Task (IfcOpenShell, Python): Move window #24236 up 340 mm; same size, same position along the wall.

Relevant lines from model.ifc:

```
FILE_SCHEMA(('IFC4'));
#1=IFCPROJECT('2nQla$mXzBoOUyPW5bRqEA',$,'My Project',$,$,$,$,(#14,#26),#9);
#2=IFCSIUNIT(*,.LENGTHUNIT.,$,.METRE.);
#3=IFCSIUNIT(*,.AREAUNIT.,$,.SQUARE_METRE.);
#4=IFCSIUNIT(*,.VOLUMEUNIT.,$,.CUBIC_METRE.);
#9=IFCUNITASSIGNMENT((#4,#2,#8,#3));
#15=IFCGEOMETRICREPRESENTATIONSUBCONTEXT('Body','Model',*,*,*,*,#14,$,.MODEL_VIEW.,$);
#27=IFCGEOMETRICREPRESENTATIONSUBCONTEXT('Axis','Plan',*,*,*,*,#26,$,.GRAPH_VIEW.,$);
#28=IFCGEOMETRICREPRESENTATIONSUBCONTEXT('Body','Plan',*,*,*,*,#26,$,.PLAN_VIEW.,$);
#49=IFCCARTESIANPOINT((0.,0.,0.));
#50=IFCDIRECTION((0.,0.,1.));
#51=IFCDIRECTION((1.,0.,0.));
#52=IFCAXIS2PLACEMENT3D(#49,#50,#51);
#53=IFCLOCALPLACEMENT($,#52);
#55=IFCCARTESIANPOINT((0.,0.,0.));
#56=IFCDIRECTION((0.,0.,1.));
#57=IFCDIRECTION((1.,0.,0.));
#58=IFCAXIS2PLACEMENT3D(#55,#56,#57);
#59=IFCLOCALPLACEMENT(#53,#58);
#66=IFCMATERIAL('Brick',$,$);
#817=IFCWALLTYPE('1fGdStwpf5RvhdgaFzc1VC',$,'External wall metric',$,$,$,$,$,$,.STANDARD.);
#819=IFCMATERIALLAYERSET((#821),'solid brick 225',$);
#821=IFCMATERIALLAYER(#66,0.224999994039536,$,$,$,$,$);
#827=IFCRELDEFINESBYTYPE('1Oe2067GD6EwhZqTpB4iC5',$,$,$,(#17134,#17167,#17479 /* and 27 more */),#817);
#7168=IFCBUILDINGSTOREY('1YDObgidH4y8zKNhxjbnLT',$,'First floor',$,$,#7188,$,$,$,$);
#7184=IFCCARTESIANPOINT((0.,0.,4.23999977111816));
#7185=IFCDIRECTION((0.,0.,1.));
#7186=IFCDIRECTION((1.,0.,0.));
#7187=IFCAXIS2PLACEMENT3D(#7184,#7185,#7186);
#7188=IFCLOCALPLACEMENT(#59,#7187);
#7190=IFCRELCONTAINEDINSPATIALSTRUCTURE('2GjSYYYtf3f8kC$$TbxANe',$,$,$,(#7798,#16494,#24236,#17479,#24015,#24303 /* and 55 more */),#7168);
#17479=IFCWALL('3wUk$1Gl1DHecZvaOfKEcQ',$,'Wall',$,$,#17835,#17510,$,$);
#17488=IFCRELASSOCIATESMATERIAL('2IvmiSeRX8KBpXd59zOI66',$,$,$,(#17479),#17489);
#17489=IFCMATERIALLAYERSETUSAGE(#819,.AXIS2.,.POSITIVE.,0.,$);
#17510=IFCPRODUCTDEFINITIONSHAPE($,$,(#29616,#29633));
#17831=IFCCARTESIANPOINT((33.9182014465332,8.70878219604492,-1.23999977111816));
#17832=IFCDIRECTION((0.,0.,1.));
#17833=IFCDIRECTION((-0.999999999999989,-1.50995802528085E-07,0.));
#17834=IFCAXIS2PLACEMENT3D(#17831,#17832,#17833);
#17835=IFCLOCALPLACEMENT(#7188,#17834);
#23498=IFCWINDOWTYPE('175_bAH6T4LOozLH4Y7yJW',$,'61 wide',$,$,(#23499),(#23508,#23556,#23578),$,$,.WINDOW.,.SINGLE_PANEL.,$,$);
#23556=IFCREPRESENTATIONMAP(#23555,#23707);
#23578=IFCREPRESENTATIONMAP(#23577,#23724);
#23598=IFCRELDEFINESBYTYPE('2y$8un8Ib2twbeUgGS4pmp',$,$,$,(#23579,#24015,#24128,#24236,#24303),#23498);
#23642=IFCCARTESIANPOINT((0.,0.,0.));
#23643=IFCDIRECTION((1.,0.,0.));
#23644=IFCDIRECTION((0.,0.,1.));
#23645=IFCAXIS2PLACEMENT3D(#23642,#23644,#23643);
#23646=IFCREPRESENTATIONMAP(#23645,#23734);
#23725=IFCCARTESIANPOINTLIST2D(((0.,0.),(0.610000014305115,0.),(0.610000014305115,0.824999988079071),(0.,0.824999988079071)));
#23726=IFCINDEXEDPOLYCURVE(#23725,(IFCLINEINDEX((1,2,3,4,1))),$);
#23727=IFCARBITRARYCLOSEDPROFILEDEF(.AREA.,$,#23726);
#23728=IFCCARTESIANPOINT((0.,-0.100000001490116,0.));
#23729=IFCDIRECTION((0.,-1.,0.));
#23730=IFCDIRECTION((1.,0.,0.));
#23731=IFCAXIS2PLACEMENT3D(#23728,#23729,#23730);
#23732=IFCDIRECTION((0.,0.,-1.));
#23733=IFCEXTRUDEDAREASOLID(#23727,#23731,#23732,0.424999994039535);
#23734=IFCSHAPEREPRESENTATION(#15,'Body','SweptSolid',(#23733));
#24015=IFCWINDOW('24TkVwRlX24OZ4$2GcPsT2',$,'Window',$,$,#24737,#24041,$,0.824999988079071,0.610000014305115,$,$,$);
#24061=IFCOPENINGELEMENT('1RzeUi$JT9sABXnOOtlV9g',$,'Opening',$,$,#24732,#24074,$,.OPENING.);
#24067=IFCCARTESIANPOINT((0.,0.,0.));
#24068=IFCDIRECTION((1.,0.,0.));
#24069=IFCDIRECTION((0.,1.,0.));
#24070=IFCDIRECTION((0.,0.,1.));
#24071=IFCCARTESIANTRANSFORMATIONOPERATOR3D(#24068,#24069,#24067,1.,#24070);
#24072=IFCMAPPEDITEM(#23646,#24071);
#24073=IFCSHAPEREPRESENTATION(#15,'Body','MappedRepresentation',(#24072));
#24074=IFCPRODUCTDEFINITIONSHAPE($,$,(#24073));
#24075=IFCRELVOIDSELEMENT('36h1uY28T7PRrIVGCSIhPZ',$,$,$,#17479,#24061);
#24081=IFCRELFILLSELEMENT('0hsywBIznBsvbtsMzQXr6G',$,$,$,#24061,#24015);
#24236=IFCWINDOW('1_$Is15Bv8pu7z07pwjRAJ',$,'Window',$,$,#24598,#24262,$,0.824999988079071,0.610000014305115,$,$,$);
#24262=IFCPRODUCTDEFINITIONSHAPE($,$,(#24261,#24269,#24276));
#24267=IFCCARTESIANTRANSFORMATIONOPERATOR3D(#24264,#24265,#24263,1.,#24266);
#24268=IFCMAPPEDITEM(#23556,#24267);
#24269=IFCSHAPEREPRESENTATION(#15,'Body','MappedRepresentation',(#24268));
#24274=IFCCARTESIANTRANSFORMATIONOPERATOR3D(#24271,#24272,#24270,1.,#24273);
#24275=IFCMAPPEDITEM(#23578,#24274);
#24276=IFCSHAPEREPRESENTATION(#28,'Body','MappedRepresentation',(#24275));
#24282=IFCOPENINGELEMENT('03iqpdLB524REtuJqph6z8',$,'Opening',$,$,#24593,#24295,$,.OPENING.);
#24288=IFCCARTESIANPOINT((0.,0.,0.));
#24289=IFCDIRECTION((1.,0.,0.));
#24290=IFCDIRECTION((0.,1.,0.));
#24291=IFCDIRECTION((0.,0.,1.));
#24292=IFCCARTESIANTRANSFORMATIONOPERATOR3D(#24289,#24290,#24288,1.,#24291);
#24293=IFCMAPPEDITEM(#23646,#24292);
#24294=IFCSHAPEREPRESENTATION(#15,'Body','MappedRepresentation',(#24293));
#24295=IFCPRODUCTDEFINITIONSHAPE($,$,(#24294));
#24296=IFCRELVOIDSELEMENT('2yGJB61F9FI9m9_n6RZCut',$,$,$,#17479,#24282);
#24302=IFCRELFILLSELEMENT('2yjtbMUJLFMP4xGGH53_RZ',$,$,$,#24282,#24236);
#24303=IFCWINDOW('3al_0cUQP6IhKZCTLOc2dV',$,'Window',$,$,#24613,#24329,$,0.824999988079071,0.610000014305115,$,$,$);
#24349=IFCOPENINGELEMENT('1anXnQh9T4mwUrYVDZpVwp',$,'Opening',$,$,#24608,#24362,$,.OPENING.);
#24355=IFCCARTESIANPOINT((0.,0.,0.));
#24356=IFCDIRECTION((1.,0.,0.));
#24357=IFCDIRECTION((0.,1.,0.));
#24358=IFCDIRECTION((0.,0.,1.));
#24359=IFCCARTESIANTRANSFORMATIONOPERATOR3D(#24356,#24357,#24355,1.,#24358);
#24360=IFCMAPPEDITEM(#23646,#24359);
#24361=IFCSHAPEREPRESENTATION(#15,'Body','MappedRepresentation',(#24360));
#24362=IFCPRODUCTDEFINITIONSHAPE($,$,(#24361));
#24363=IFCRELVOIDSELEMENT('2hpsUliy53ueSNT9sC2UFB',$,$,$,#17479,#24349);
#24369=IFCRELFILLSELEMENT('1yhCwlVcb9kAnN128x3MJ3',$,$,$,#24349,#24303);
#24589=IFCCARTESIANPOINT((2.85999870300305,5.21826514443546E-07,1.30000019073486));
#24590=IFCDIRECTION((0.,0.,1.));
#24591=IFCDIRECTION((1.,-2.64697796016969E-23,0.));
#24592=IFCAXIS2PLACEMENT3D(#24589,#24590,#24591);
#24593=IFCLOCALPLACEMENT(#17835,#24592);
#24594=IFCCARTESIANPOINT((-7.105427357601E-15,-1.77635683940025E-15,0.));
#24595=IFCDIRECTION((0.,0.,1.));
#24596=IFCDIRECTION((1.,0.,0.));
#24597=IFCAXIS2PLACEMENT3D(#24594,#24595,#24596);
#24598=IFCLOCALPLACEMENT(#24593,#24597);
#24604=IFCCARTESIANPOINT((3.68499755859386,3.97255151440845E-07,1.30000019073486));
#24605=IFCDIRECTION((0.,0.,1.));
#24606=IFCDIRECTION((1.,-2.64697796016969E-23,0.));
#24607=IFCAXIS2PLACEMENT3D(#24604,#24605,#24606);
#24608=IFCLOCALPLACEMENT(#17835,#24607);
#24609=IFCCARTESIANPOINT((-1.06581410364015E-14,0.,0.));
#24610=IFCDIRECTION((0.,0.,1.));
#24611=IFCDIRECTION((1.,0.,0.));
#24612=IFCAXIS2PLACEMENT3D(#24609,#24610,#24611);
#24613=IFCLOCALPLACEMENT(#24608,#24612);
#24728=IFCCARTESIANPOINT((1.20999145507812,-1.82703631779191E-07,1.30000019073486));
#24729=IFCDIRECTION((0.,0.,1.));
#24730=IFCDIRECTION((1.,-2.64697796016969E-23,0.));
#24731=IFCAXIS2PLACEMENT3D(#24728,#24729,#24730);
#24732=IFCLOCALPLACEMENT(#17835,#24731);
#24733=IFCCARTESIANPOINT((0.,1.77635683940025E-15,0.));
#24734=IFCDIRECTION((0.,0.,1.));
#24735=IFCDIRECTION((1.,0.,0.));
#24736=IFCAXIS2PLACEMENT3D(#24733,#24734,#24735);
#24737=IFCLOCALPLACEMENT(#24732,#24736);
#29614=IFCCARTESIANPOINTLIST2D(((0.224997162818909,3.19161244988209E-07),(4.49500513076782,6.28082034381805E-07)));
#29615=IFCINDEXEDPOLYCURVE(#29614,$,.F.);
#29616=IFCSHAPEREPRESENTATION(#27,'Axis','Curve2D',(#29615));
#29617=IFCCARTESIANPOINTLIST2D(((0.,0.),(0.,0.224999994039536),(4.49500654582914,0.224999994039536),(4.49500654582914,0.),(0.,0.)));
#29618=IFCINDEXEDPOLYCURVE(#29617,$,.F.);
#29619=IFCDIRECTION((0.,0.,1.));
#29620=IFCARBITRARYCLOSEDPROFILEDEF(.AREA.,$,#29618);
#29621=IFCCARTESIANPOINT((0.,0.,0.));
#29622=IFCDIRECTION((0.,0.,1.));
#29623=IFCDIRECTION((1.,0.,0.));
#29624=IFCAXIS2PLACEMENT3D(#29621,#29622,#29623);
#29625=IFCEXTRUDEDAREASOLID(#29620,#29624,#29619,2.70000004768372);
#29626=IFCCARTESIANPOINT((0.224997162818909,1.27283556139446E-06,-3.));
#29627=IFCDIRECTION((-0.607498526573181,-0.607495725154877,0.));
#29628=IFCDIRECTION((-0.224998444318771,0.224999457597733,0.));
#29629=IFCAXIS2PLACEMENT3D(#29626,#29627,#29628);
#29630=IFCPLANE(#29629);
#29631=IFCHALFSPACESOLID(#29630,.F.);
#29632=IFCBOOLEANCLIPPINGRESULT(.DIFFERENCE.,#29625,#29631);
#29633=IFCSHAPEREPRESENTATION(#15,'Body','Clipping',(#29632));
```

```python
import numpy as np
import ifcopenshell
import ifcopenshell.api.geometry
import ifcopenshell.util.placement
import ifcopenshell.util.unit

model = ifcopenshell.open("model.ifc")
unit_scale = ifcopenshell.util.unit.calculate_unit_scale(model)

window = model.by_guid("1_$Is15Bv8pu7z07pwjRAJ")
opening = window.FillsVoids[0].RelatingOpeningElement
dz = 0.34

shift = np.array([0.0, 0.0, dz])
# The window is placed relative to its opening, so it follows when the opening moves.
matrix = ifcopenshell.util.placement.get_local_placement(opening.ObjectPlacement)
matrix[:3, 3] += shift
ifcopenshell.api.geometry.edit_object_placement(
    model, product=opening, matrix=matrix, is_si=False, should_transform_children=True
)

print(f"moved by {dz * unit_scale:+.3f} m")

model.write("model-out.ifc")
```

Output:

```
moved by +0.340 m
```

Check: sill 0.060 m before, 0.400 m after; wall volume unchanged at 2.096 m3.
